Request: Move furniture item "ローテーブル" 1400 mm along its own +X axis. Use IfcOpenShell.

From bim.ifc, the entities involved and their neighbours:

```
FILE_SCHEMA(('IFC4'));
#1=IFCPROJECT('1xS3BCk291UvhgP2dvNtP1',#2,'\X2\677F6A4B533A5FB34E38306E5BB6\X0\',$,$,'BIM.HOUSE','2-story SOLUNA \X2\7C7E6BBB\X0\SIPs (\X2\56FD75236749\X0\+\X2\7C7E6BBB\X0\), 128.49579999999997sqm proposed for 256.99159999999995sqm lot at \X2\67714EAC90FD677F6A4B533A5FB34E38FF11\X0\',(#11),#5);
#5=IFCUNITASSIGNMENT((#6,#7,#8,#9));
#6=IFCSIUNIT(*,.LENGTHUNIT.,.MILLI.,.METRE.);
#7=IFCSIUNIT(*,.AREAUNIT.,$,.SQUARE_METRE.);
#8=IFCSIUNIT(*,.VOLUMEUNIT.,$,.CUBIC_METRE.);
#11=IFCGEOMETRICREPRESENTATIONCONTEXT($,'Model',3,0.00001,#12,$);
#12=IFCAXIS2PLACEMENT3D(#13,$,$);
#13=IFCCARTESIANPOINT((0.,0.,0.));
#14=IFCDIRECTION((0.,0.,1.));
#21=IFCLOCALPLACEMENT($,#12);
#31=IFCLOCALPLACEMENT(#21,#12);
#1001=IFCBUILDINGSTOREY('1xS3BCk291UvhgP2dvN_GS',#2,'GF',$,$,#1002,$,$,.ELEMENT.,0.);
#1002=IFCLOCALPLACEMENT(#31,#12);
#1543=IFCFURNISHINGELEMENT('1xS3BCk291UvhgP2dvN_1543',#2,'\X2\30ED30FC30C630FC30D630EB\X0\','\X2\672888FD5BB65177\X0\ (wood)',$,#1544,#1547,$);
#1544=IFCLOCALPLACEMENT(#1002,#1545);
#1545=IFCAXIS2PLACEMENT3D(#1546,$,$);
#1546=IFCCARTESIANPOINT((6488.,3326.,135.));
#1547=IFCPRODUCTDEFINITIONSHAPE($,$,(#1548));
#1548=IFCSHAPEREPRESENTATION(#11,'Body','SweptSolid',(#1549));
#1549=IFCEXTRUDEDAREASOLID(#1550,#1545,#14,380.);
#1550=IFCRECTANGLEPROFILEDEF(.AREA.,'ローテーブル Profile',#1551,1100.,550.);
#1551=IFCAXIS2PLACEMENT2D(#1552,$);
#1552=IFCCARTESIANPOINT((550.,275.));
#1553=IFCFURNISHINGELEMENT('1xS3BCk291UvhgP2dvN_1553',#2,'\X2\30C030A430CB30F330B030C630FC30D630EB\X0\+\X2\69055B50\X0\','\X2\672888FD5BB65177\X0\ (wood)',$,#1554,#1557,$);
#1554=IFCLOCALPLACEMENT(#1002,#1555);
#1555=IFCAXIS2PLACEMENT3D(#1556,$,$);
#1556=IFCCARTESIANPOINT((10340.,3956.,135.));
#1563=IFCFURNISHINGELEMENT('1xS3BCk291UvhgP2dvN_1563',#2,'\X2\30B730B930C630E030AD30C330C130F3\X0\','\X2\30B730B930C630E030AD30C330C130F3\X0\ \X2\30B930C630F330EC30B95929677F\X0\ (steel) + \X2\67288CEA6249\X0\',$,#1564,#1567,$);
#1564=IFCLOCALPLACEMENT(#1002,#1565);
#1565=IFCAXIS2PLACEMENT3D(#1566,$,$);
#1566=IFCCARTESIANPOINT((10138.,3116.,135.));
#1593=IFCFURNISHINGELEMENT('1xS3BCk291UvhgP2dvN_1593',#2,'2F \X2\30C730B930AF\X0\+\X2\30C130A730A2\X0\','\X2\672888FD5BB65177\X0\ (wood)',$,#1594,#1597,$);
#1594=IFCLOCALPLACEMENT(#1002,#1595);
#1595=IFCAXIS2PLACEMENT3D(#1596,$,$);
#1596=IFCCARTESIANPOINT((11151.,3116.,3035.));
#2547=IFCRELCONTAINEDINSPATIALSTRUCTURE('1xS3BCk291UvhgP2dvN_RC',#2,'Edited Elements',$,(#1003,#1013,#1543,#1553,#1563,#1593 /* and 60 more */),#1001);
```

```python
import ifcopenshell
import ifcopenshell.api.geometry
import ifcopenshell.util.placement

model = ifcopenshell.open("bim.ifc")

item = model.by_guid("1xS3BCk291UvhgP2dvN_1543")
matrix = ifcopenshell.util.placement.get_local_placement(item.ObjectPlacement)
matrix[:3, 3] += matrix[:3, 0] * 1400.0
ifcopenshell.api.geometry.edit_object_placement(model, product=item, matrix=matrix, is_si=False)

print(ifcopenshell.util.placement.get_local_placement(item.ObjectPlacement).round(3) + 0.0)

model.write("bim_updated.ifc")
```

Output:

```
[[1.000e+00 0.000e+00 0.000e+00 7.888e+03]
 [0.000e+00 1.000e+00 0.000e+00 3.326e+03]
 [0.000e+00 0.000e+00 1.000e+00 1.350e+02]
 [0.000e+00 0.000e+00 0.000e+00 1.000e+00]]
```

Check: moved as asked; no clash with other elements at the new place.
